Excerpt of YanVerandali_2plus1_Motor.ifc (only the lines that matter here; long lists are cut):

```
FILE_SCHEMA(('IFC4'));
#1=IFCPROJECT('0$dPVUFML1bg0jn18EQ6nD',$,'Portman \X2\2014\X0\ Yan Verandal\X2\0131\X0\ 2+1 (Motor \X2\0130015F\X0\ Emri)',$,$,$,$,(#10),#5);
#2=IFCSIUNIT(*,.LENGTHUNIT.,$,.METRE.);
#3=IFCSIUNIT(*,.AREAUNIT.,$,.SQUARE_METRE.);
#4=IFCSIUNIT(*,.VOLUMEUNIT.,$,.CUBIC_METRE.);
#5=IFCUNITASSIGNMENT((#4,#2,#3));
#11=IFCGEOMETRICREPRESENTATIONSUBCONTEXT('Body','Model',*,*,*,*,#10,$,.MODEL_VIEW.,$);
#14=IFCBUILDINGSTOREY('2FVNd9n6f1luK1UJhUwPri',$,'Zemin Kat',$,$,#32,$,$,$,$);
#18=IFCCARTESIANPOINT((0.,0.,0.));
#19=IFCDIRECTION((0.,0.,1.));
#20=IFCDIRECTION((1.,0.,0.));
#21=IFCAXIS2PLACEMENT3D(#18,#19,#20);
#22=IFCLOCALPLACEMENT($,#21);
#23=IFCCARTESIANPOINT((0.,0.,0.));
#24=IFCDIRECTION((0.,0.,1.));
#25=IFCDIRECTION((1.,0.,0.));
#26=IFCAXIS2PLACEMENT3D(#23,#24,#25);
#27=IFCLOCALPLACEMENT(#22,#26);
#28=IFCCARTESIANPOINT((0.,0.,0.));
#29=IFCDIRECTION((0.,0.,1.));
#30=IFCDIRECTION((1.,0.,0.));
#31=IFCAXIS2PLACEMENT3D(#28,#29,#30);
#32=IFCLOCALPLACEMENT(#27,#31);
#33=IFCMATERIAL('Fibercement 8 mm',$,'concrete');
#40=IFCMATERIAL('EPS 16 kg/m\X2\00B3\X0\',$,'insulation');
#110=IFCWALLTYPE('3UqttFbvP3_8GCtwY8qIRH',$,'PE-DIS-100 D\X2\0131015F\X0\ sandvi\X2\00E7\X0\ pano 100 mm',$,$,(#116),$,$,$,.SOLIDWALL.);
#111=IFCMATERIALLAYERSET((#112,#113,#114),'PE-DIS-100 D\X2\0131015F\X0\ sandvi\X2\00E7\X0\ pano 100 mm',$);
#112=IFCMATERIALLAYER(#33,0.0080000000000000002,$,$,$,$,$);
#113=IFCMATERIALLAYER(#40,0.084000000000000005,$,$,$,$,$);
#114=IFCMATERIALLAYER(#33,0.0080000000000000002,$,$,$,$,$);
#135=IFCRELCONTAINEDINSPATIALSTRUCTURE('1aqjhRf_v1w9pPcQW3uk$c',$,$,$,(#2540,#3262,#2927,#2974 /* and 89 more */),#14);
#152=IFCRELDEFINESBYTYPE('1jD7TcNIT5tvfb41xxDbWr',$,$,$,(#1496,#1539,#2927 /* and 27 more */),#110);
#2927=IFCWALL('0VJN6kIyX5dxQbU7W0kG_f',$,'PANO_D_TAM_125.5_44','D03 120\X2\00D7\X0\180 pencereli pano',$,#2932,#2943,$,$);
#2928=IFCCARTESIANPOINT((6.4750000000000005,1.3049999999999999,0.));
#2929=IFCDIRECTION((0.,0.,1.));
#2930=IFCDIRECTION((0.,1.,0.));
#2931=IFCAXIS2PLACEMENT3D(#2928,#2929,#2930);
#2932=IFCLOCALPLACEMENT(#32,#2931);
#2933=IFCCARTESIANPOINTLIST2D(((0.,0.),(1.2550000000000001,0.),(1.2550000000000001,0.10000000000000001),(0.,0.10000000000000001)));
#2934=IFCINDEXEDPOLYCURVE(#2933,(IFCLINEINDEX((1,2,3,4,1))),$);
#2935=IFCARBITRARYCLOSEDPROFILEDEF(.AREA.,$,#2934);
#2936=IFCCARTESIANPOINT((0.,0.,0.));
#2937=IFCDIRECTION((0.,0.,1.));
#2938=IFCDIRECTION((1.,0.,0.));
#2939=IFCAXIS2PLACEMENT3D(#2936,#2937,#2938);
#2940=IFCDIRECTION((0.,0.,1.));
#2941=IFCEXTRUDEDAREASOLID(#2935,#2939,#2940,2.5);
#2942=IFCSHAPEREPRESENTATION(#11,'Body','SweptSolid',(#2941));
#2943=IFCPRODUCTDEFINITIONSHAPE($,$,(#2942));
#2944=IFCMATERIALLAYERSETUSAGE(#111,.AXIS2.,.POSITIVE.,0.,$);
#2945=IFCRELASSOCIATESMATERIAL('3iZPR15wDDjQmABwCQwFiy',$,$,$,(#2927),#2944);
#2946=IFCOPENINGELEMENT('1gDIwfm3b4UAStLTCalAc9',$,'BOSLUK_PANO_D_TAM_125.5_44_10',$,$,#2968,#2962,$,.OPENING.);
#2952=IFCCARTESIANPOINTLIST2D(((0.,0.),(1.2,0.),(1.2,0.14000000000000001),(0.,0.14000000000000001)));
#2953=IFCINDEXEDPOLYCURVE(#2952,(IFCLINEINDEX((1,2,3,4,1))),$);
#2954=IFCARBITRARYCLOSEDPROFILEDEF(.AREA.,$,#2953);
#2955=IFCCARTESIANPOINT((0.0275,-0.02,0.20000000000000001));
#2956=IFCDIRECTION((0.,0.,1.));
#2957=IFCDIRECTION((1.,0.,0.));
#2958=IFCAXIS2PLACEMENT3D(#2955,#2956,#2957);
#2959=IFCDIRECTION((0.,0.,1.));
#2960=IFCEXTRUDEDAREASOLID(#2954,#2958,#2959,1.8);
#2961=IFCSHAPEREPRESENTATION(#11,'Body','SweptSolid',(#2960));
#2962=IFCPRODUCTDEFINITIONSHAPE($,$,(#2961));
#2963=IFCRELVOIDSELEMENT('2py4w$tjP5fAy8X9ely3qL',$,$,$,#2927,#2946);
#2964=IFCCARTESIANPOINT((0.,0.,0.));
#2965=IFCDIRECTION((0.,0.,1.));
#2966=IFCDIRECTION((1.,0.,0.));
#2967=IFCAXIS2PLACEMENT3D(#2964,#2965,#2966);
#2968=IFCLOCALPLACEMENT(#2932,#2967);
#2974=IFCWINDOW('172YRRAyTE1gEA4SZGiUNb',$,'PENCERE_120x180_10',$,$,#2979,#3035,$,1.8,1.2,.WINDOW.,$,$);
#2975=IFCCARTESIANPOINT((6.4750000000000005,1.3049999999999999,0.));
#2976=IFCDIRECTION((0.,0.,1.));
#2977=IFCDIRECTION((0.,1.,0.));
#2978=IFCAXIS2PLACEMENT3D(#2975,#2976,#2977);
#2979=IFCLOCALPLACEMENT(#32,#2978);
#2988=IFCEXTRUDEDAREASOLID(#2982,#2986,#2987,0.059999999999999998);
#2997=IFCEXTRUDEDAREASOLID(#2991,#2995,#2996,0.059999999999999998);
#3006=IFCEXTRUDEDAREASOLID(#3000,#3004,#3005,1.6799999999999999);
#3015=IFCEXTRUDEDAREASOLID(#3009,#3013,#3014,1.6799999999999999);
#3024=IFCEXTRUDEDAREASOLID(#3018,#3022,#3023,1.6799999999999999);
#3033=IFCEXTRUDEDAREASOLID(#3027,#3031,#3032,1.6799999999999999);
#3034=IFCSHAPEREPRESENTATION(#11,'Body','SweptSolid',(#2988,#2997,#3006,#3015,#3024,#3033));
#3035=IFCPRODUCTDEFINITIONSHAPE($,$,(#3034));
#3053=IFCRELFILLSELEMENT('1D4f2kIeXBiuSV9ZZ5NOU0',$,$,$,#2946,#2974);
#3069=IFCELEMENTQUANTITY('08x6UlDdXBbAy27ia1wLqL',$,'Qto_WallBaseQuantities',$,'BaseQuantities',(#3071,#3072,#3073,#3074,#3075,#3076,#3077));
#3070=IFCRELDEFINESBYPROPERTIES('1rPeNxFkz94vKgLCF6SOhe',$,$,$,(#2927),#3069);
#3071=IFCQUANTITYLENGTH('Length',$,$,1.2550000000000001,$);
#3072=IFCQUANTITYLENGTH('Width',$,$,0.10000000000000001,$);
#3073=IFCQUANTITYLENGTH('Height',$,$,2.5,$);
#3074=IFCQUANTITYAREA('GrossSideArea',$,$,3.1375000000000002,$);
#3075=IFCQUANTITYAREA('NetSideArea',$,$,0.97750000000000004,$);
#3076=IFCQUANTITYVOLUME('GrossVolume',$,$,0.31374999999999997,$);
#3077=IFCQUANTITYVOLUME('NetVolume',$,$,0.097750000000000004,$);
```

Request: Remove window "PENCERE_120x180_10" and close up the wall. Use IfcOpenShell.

```python
import ifcopenshell
import ifcopenshell.api.feature
import ifcopenshell.api.pset
import ifcopenshell.api.root
import ifcopenshell.geom
import ifcopenshell.util.element
import ifcopenshell.util.shape
import ifcopenshell.util.unit

model = ifcopenshell.open("YanVerandali_2plus1_Motor.ifc")
area_scale = ifcopenshell.util.unit.calculate_unit_scale(model, "AREAUNIT")
volume_scale = ifcopenshell.util.unit.calculate_unit_scale(model, "VOLUMEUNIT")
settings = ifcopenshell.geom.settings()


def volume(element):
    """Net volume in cubic metres, openings subtracted."""
    shape = ifcopenshell.geom.create_shape(settings, element)
    return ifcopenshell.util.shape.get_volume(shape.geometry)


window = model.by_guid("172YRRAyTE1gEA4SZGiUNb")
opening = window.FillsVoids[0].RelatingOpeningElement
wall = opening.VoidsElements[0].RelatingBuildingElement
before = volume(wall)

ifcopenshell.api.root.remove_product(model, product=window)
ifcopenshell.api.feature.remove_feature(model, feature=opening)

after = volume(wall)
thickness = 0.1  # wall thickness in metres

# Update the wall's stored quantities.
qto = model.by_id(ifcopenshell.util.element.get_pset(wall, "Qto_WallBaseQuantities", should_inherit=False)["id"])
ifcopenshell.api.pset.edit_qto(model, qto=qto, properties={
    "NetSideArea": after / thickness / area_scale,
    "NetVolume": after / volume_scale,
})

print(f"wall volume {before:.3f} -> {after:.3f} m3")

model.write("YanVerandali_2plus1_Motor_rev.ifc")
```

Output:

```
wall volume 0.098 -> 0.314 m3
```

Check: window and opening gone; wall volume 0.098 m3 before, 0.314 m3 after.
